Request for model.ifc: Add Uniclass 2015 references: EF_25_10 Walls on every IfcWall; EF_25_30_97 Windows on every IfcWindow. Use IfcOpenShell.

First a look at what the model holds.

```python
import ifcopenshell

model = ifcopenshell.open("model.ifc")
print(model.schema)
print("classifications:", [c.Name for c in model.by_type("IfcClassification")])
for ifc_class in ("IfcDoor", "IfcRoof", "IfcStair", "IfcWall", "IfcWindow"):
    print(ifc_class, len(model.by_type(ifc_class)))
```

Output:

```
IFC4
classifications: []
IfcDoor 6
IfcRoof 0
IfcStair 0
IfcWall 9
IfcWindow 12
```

```python
import ifcopenshell
import ifcopenshell.api.classification

model = ifcopenshell.open("model.ifc")

system = ifcopenshell.api.classification.add_classification(model, classification="Uniclass 2015")

codes = {
    "IfcWall": ("EF_25_10", "Walls"),
    "IfcWindow": ("EF_25_30_97", "Windows"),
}
for ifc_class, (code, name) in codes.items():
    products = model.by_type(ifc_class)
    ifcopenshell.api.classification.add_reference(
        model, products=products, classification=system, identification=code, name=name
    )
    print(code, len(products))

model.write("model_updated.ifc")
```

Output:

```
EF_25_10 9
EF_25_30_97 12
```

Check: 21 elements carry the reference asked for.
